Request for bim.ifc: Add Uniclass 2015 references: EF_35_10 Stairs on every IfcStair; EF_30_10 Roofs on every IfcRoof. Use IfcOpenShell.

First a look at what the model holds.

```python
import ifcopenshell

model = ifcopenshell.open("bim.ifc")
print(model.schema)
print("classifications:", [c.Name for c in model.by_type("IfcClassification")])
for ifc_class in ("IfcDoor", "IfcRoof", "IfcStair", "IfcWall", "IfcWindow"):
    print(ifc_class, len(model.by_type(ifc_class)))
```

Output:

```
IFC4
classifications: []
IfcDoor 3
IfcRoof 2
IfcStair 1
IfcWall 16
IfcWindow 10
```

```python
import ifcopenshell
import ifcopenshell.api.classification

model = ifcopenshell.open("bim.ifc")

system = ifcopenshell.api.classification.add_classification(model, classification="Uniclass 2015")

codes = {
    "IfcStair": ("EF_35_10", "Stairs"),
    "IfcRoof": ("EF_30_10", "Roofs"),
}
for ifc_class, (code, name) in codes.items():
    products = model.by_type(ifc_class)
    ifcopenshell.api.classification.add_reference(
        model, products=products, classification=system, identification=code, name=name
    )
    print(code, len(products))

model.write("bim_rev.ifc")
```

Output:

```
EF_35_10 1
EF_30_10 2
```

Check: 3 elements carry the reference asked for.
